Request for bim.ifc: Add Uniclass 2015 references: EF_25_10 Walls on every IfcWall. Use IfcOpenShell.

First a look at what the model holds.

```python
import ifcopenshell

model = ifcopenshell.open("bim.ifc")
print(model.schema)
print("classifications:", [c.Name for c in model.by_type("IfcClassification")])
for ifc_class in ("IfcDoor", "IfcRoof", "IfcStair", "IfcWall", "IfcWindow"):
    print(ifc_class, len(model.by_type(ifc_class)))
```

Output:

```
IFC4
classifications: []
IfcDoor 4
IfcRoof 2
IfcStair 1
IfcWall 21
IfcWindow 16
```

```python
import ifcopenshell
import ifcopenshell.api.classification

model = ifcopenshell.open("bim.ifc")

system = ifcopenshell.api.classification.add_classification(model, classification="Uniclass 2015")

codes = {
    "IfcWall": ("EF_25_10", "Walls"),
}
for ifc_class, (code, name) in codes.items():
    products = model.by_type(ifc_class)
    ifcopenshell.api.classification.add_reference(
        model, products=products, classification=system, identification=code, name=name
    )
    print(code, len(products))

model.write("bim_v2.ifc")
```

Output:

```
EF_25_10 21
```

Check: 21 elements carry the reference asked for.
